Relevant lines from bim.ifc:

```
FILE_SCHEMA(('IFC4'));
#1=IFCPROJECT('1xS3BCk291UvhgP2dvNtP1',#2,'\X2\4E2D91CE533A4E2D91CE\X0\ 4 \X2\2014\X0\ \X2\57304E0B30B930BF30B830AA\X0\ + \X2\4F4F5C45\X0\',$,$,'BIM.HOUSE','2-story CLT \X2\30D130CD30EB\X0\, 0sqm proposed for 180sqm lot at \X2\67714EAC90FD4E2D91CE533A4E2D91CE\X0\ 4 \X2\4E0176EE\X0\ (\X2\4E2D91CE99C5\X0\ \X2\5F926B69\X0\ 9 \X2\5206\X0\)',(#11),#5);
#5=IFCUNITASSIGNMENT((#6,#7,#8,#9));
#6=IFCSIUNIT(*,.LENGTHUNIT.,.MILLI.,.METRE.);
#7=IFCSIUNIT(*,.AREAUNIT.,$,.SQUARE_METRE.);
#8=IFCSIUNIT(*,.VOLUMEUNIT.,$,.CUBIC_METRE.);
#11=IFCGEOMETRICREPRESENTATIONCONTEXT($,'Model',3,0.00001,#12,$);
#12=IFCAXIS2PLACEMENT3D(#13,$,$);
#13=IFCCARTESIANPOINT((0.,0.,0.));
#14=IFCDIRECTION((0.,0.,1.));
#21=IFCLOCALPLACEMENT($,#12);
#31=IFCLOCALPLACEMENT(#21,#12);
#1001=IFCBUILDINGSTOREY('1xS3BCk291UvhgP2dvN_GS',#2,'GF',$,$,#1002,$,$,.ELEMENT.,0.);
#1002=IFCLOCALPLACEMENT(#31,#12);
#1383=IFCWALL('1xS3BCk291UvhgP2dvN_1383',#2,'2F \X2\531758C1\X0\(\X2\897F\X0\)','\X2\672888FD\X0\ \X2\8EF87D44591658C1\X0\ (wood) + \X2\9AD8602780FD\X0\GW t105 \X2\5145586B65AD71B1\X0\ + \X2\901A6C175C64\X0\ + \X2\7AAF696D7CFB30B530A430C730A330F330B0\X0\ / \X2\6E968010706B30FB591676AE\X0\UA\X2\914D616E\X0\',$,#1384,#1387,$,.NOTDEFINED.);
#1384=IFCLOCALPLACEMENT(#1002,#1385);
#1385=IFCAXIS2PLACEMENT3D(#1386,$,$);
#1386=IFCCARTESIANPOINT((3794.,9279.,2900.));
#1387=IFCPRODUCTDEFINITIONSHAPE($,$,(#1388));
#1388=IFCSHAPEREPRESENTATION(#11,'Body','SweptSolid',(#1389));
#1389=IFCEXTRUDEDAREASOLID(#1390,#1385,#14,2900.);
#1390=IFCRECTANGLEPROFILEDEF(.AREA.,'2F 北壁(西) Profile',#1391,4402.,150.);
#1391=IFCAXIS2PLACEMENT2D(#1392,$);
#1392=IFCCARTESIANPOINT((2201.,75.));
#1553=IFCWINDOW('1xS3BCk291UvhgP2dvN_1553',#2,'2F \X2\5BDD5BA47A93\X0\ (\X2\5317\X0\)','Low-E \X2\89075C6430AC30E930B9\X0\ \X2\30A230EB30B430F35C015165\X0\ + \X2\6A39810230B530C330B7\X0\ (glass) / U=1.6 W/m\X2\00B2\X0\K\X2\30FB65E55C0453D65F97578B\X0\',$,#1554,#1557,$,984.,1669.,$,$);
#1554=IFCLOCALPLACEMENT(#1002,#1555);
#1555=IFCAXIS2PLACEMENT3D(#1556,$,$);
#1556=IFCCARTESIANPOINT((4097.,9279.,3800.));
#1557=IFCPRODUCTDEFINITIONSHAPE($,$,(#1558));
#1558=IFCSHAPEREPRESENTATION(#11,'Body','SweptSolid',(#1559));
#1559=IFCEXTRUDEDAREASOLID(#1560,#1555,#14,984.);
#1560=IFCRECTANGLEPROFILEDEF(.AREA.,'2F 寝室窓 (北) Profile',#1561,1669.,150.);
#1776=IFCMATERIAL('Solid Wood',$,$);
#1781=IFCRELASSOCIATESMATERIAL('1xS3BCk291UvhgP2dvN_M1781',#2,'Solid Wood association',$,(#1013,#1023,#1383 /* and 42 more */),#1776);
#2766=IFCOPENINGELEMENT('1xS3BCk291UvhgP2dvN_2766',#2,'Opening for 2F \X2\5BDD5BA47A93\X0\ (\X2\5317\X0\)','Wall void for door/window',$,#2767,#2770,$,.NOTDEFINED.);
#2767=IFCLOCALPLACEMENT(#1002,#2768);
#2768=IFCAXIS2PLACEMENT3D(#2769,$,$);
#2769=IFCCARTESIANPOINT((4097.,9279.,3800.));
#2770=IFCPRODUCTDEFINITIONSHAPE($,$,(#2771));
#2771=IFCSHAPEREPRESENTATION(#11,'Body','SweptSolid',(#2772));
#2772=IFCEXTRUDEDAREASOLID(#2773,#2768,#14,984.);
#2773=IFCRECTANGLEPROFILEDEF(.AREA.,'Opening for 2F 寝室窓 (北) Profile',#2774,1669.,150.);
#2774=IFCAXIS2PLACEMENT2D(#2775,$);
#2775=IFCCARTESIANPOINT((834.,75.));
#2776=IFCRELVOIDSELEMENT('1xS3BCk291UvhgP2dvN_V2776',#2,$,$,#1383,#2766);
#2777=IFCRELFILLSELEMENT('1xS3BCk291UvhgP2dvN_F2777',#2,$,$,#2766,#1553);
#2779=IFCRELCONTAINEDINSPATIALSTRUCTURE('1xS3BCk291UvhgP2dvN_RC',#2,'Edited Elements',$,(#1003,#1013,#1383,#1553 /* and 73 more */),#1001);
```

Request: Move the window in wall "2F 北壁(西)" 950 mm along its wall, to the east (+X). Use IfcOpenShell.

```python
import ifcopenshell
import ifcopenshell.api.geometry
import ifcopenshell.util.placement
import ifcopenshell.util.unit

model = ifcopenshell.open("bim.ifc")
unit_scale = ifcopenshell.util.unit.calculate_unit_scale(model)

window = model.by_id(1553)
opening = window.FillsVoids[0].RelatingOpeningElement
wall = opening.VoidsElements[0].RelatingBuildingElement

wall_matrix = ifcopenshell.util.placement.get_local_placement(wall.ObjectPlacement)
shift = wall_matrix[:3, 0] * 0.95 / unit_scale
before = ifcopenshell.util.placement.get_local_placement(window.ObjectPlacement)[:3, 3].copy()

# The window is not placed relative to its opening, so move both.
for product in (opening, window):
    matrix = ifcopenshell.util.placement.get_local_placement(product.ObjectPlacement)
    matrix[:3, 3] += shift
    ifcopenshell.api.geometry.edit_object_placement(model, product=product, matrix=matrix, is_si=False)

after = ifcopenshell.util.placement.get_local_placement(window.ObjectPlacement)[:3, 3]
print("window moved by", (after - before).round(3) + 0.0)

model.write("bim_v2.ifc")
```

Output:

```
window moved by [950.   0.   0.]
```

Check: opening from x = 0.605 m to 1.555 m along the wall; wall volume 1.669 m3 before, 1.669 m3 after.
